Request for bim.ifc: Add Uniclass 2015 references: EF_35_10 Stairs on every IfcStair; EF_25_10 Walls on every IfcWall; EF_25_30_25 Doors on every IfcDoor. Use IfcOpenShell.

First a look at what the model holds.

```python
import ifcopenshell

model = ifcopenshell.open("bim.ifc")
print(model.schema)
print("classifications:", [c.Name for c in model.by_type("IfcClassification")])
for ifc_class in ("IfcDoor", "IfcRoof", "IfcStair", "IfcWall", "IfcWindow"):
    print(ifc_class, len(model.by_type(ifc_class)))
```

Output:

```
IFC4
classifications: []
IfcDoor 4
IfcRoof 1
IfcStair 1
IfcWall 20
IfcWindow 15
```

```python
import ifcopenshell
import ifcopenshell.api.classification

model = ifcopenshell.open("bim.ifc")

system = ifcopenshell.api.classification.add_classification(model, classification="Uniclass 2015")

codes = {
    "IfcStair": ("EF_35_10", "Stairs"),
    "IfcWall": ("EF_25_10", "Walls"),
    "IfcDoor": ("EF_25_30_25", "Doors"),
}
for ifc_class, (code, name) in codes.items():
    products = model.by_type(ifc_class)
    ifcopenshell.api.classification.add_reference(
        model, products=products, classification=system, identification=code, name=name
    )
    print(code, len(products))

model.write("bim_v2.ifc")
```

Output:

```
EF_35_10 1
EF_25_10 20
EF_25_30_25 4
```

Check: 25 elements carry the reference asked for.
